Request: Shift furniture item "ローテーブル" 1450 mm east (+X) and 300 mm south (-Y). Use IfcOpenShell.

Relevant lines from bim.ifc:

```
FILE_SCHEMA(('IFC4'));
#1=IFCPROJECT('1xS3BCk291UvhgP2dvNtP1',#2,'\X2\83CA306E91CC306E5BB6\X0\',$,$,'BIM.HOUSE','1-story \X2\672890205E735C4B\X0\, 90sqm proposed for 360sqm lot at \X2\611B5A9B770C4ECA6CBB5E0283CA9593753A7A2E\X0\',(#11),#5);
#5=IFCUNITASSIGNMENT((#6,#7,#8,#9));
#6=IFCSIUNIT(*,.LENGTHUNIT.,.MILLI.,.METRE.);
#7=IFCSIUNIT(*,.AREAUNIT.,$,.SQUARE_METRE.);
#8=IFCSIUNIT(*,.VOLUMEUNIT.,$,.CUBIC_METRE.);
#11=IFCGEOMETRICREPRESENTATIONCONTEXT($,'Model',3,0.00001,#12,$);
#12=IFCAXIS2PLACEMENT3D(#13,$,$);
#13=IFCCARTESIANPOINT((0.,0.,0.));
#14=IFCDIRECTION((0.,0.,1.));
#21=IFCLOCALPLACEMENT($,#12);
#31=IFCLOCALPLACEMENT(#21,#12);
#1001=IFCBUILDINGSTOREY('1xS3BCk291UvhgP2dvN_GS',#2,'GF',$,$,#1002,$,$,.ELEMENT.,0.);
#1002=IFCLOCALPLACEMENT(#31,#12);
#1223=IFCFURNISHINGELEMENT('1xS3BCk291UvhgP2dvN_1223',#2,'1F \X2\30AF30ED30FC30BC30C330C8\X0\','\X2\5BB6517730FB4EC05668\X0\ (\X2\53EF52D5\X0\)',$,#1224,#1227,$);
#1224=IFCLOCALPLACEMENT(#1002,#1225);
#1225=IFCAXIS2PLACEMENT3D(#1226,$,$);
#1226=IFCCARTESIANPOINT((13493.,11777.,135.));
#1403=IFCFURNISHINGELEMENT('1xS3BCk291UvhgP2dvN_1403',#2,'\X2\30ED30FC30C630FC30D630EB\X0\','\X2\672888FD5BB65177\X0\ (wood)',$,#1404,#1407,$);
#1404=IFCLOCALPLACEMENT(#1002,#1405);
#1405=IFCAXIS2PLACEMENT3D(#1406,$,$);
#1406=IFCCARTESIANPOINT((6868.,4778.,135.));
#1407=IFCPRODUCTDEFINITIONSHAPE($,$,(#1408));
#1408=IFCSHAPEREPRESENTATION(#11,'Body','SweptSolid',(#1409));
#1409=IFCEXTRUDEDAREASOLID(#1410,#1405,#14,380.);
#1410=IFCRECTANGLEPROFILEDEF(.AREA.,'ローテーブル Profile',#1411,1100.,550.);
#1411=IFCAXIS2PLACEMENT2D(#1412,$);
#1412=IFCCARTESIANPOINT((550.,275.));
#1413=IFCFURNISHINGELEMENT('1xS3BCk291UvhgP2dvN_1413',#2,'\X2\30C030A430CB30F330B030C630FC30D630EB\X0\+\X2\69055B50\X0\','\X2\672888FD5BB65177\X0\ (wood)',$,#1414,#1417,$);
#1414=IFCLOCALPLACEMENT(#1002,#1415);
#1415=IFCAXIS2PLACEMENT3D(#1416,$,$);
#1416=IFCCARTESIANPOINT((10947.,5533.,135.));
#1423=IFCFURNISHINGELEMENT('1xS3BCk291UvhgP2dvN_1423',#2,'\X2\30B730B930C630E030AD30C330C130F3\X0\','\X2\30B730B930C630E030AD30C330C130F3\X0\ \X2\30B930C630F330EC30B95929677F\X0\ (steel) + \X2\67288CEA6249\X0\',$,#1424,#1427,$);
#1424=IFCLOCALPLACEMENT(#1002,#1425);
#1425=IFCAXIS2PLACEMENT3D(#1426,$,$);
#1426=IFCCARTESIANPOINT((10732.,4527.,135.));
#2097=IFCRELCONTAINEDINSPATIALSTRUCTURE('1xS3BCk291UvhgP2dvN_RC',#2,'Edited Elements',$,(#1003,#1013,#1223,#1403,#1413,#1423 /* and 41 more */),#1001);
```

```python
import ifcopenshell
import ifcopenshell.api.geometry
import ifcopenshell.util.placement

model = ifcopenshell.open("bim.ifc")

item = model.by_id(1403)
matrix = ifcopenshell.util.placement.get_local_placement(item.ObjectPlacement)
matrix[0, 3] += 1450.0
matrix[1, 3] -= 300.0
ifcopenshell.api.geometry.edit_object_placement(model, product=item, matrix=matrix, is_si=False)

print(ifcopenshell.util.placement.get_local_placement(item.ObjectPlacement).round(3) + 0.0)

model.write("bim_updated.ifc")
```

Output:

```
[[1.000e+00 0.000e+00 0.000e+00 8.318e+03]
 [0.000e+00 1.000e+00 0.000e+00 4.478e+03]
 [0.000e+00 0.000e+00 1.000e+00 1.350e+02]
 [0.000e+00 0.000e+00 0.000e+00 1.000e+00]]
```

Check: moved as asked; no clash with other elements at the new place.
